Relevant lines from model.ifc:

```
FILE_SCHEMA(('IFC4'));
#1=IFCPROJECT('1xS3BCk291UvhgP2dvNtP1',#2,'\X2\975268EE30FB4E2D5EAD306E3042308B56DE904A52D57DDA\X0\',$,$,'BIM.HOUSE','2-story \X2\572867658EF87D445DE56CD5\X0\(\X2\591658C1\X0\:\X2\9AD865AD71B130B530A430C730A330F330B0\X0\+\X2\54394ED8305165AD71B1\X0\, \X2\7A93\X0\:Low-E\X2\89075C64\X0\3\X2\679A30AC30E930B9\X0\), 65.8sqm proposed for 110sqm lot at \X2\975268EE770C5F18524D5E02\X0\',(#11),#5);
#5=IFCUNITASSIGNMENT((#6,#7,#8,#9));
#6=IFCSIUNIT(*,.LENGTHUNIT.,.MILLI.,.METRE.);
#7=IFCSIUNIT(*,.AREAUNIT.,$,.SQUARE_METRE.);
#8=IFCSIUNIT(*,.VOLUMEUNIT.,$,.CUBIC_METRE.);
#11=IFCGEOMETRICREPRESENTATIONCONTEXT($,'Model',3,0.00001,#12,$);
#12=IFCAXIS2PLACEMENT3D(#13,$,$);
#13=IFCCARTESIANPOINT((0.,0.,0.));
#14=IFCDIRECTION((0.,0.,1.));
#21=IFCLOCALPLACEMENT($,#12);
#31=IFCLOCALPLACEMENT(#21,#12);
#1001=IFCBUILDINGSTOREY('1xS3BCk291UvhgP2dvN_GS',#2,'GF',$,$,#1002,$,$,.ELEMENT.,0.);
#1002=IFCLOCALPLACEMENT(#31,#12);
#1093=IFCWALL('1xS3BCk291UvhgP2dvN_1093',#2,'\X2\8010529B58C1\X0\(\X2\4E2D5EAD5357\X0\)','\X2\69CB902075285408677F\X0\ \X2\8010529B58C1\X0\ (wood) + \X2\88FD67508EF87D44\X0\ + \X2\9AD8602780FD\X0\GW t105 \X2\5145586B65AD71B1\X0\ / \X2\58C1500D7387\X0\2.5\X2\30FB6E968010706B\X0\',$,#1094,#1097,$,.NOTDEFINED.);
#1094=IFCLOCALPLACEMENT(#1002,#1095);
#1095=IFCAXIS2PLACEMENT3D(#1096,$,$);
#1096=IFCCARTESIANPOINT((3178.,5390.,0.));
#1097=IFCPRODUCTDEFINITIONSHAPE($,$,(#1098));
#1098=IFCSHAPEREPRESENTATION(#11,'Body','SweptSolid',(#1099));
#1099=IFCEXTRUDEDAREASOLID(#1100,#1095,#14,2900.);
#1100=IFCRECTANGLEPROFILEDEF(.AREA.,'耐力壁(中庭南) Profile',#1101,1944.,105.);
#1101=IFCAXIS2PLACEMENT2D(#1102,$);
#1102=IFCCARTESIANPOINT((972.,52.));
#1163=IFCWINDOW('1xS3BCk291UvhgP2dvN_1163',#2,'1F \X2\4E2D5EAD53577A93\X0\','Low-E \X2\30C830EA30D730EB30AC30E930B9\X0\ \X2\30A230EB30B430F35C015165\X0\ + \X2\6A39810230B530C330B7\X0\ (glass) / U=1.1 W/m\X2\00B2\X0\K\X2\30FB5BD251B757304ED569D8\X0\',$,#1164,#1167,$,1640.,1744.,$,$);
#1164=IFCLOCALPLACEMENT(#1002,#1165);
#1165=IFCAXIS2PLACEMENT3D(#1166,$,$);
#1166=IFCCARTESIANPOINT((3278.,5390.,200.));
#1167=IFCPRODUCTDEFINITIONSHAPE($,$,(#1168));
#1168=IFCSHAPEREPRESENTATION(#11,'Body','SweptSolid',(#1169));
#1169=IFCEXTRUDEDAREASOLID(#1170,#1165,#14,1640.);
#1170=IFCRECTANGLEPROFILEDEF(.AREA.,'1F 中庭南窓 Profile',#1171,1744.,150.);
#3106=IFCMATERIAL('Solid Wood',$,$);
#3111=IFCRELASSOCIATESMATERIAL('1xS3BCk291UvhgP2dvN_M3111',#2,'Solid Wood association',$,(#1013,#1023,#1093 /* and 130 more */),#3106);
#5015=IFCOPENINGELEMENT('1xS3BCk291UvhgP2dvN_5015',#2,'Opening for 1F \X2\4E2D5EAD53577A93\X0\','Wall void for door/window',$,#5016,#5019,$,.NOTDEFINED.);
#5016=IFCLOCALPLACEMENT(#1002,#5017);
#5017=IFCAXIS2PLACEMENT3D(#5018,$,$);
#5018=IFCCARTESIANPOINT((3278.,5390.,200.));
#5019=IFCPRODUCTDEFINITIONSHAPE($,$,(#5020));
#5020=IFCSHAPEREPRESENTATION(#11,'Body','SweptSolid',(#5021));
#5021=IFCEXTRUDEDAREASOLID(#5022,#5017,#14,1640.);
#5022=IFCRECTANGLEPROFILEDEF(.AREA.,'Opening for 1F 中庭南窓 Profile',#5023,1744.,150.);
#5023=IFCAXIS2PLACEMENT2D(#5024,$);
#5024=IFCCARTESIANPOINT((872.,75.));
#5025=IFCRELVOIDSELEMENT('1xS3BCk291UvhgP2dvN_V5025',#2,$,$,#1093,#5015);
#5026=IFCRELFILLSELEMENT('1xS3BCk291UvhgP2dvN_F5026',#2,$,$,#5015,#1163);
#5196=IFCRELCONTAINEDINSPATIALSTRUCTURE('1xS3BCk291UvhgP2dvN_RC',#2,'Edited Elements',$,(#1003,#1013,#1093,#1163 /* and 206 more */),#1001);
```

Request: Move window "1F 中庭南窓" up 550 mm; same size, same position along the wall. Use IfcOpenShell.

```python
import numpy as np
import ifcopenshell
import ifcopenshell.api.geometry
import ifcopenshell.util.placement
import ifcopenshell.util.unit

model = ifcopenshell.open("model.ifc")
unit_scale = ifcopenshell.util.unit.calculate_unit_scale(model)

window = model.by_guid("1xS3BCk291UvhgP2dvN_1163")
opening = window.FillsVoids[0].RelatingOpeningElement
dz = 550.0

shift = np.array([0.0, 0.0, dz])
# The window is not placed relative to its opening, so move both.
for product in (opening, window):
    matrix = ifcopenshell.util.placement.get_local_placement(product.ObjectPlacement)
    matrix[:3, 3] += shift
    ifcopenshell.api.geometry.edit_object_placement(model, product=product, matrix=matrix, is_si=False)

print(f"moved by {dz * unit_scale:+.3f} m")

model.write("model_edited.ifc")
```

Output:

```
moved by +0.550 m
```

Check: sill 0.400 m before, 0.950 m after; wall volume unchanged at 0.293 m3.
